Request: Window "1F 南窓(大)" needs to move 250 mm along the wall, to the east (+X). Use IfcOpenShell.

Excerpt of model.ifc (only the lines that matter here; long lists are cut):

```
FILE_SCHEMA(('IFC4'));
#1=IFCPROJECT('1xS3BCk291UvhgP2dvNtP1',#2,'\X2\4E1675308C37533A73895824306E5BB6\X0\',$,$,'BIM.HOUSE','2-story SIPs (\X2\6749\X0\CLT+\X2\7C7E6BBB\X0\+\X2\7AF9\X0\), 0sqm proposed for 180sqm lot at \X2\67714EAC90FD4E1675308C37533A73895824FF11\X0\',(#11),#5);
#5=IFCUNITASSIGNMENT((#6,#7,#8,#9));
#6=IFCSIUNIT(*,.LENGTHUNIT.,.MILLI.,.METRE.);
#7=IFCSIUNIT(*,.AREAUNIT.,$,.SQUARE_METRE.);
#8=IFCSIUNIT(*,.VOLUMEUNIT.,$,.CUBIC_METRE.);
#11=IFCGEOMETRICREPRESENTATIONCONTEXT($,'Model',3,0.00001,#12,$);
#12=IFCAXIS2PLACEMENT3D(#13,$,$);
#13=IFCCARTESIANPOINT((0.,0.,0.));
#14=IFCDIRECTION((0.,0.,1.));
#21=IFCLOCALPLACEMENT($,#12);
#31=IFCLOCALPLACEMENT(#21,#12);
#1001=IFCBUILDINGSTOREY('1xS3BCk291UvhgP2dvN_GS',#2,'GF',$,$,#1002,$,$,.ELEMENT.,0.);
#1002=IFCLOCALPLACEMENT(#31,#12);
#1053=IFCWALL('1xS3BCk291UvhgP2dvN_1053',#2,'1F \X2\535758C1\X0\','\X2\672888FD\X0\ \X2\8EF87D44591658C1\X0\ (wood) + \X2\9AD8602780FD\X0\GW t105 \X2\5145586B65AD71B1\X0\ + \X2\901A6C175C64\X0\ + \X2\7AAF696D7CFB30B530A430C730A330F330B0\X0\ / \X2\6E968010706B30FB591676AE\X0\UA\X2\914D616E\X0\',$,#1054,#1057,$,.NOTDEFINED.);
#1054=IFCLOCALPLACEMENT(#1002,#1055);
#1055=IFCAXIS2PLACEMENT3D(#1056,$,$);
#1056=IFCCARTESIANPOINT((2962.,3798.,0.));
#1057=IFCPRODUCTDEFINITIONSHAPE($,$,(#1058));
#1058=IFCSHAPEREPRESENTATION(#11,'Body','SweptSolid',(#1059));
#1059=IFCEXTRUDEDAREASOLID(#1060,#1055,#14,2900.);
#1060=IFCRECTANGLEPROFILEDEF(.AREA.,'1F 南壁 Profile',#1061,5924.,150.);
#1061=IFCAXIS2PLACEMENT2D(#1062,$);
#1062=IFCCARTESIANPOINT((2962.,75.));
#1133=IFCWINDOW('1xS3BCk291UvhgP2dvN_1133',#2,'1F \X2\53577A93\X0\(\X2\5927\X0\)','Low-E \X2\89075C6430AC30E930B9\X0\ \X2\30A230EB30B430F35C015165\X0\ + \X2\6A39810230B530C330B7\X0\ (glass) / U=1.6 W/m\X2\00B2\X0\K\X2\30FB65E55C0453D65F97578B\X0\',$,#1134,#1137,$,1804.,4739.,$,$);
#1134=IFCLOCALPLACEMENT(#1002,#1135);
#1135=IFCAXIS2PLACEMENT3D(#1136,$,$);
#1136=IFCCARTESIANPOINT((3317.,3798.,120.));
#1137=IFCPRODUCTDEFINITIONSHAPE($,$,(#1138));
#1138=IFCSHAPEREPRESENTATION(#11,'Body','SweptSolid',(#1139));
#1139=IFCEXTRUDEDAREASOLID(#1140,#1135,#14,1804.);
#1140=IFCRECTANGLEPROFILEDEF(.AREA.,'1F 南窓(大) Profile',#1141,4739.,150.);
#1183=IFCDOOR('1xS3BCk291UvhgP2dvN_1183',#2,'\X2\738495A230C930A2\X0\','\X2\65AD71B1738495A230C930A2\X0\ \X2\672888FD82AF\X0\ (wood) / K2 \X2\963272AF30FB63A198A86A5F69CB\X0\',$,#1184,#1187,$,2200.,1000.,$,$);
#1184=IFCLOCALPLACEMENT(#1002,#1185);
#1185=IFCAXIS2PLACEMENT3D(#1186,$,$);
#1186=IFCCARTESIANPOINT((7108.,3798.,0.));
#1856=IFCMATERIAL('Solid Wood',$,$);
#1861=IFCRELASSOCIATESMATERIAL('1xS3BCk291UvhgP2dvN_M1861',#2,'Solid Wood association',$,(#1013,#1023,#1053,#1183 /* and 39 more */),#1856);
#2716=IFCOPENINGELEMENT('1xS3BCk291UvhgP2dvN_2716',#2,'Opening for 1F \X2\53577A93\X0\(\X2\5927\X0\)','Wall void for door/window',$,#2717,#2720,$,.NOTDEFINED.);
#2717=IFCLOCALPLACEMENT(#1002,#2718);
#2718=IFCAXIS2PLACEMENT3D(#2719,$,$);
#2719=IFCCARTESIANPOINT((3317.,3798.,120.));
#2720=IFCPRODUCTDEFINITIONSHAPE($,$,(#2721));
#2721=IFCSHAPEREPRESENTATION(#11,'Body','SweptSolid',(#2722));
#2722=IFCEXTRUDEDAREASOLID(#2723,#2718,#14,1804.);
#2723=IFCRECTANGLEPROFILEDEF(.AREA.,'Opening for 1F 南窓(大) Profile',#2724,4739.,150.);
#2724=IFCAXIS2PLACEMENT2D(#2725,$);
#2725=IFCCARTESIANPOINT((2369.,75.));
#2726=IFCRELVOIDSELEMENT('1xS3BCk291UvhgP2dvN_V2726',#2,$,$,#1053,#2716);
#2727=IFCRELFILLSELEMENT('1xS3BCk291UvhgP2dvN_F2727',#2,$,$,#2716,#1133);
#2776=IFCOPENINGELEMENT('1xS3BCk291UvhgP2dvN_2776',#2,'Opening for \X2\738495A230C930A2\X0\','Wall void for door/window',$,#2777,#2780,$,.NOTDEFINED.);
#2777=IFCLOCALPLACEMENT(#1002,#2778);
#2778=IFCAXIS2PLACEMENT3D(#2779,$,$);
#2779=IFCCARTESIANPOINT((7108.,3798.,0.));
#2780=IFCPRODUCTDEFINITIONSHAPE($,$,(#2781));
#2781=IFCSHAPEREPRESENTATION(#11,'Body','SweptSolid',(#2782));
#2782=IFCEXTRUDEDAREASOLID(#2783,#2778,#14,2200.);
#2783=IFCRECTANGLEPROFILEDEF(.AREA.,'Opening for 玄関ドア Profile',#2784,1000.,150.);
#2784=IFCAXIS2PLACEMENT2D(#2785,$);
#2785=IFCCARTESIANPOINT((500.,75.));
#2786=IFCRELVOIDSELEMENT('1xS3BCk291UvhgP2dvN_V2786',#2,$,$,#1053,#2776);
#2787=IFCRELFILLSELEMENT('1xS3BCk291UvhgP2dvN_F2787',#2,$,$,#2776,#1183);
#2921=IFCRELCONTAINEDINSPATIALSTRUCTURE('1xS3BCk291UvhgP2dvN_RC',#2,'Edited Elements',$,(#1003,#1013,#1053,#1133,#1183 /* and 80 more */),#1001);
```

```python
import ifcopenshell
import ifcopenshell.api.geometry
import ifcopenshell.util.placement
import ifcopenshell.util.unit

model = ifcopenshell.open("model.ifc")
unit_scale = ifcopenshell.util.unit.calculate_unit_scale(model)

window = model.by_id(1133)
opening = window.FillsVoids[0].RelatingOpeningElement
wall = opening.VoidsElements[0].RelatingBuildingElement

wall_matrix = ifcopenshell.util.placement.get_local_placement(wall.ObjectPlacement)
shift = wall_matrix[:3, 0] * 0.25 / unit_scale
before = ifcopenshell.util.placement.get_local_placement(window.ObjectPlacement)[:3, 3].copy()

# The window is not placed relative to its opening, so move both.
for product in (opening, window):
    matrix = ifcopenshell.util.placement.get_local_placement(product.ObjectPlacement)
    matrix[:3, 3] += shift
    ifcopenshell.api.geometry.edit_object_placement(model, product=product, matrix=matrix, is_si=False)

after = ifcopenshell.util.placement.get_local_placement(window.ObjectPlacement)[:3, 3]
print("window moved by", (after - before).round(3) + 0.0)

model.write("model-out.ifc")
```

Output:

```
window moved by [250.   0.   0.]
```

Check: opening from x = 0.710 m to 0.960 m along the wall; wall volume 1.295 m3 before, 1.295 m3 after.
